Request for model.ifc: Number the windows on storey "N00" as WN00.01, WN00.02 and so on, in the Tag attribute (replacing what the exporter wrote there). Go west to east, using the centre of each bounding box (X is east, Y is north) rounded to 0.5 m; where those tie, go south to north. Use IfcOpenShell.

First a look at what the model holds.

```python
import ifcopenshell
import ifcopenshell.util.element
import ifcopenshell.util.placement

model = ifcopenshell.open("model.ifc")
print(model.schema)
storey = next(s for s in model.by_type("IfcBuildingStorey") if s.Name == "N00")
windows = [e for e in ifcopenshell.util.element.get_decomposition(storey) if e.is_a("IfcWindow")]
for e in sorted(windows, key=lambda e: e.id()):
    origin = ifcopenshell.util.placement.get_local_placement(e.ObjectPlacement)[:3, 3]
    print(e.id(), e.Tag, e.Name, origin.round(2) + 0.0, sep=" | ")
```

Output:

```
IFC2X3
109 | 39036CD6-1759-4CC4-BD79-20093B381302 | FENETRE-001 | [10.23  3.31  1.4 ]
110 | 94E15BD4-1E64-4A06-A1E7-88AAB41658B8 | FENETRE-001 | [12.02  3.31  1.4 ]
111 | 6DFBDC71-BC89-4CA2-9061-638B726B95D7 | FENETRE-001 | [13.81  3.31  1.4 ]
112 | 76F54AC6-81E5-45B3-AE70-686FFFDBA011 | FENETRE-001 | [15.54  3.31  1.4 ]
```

```python
import ifcopenshell
import ifcopenshell.geom
import ifcopenshell.util.element
import ifcopenshell.util.shape

model = ifcopenshell.open("model.ifc")
settings = ifcopenshell.geom.settings()
settings.set("use-world-coords", True)


def centre(element):
    shape = ifcopenshell.geom.create_shape(settings, element)
    return ifcopenshell.util.shape.get_bbox_centroid(shape.geometry)


storey = next(s for s in model.by_type("IfcBuildingStorey") if s.Name == "N00")
windows = [e for e in ifcopenshell.util.element.get_decomposition(storey) if e.is_a("IfcWindow")]

# Insertion points can sit at a corner or the storey origin, so sort by the geometry (in metres).
centres = {e: centre(e) for e in windows}
windows.sort(key=lambda e: (round(centres[e][0] / 0.5), centres[e][1]))

for i, e in enumerate(windows, start=1):
    number = f"WN00.{i:02d}"
    e.Tag = number
    print(e.id(), number)

model.write("model_updated.ifc")
```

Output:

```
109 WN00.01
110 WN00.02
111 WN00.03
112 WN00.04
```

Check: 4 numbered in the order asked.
